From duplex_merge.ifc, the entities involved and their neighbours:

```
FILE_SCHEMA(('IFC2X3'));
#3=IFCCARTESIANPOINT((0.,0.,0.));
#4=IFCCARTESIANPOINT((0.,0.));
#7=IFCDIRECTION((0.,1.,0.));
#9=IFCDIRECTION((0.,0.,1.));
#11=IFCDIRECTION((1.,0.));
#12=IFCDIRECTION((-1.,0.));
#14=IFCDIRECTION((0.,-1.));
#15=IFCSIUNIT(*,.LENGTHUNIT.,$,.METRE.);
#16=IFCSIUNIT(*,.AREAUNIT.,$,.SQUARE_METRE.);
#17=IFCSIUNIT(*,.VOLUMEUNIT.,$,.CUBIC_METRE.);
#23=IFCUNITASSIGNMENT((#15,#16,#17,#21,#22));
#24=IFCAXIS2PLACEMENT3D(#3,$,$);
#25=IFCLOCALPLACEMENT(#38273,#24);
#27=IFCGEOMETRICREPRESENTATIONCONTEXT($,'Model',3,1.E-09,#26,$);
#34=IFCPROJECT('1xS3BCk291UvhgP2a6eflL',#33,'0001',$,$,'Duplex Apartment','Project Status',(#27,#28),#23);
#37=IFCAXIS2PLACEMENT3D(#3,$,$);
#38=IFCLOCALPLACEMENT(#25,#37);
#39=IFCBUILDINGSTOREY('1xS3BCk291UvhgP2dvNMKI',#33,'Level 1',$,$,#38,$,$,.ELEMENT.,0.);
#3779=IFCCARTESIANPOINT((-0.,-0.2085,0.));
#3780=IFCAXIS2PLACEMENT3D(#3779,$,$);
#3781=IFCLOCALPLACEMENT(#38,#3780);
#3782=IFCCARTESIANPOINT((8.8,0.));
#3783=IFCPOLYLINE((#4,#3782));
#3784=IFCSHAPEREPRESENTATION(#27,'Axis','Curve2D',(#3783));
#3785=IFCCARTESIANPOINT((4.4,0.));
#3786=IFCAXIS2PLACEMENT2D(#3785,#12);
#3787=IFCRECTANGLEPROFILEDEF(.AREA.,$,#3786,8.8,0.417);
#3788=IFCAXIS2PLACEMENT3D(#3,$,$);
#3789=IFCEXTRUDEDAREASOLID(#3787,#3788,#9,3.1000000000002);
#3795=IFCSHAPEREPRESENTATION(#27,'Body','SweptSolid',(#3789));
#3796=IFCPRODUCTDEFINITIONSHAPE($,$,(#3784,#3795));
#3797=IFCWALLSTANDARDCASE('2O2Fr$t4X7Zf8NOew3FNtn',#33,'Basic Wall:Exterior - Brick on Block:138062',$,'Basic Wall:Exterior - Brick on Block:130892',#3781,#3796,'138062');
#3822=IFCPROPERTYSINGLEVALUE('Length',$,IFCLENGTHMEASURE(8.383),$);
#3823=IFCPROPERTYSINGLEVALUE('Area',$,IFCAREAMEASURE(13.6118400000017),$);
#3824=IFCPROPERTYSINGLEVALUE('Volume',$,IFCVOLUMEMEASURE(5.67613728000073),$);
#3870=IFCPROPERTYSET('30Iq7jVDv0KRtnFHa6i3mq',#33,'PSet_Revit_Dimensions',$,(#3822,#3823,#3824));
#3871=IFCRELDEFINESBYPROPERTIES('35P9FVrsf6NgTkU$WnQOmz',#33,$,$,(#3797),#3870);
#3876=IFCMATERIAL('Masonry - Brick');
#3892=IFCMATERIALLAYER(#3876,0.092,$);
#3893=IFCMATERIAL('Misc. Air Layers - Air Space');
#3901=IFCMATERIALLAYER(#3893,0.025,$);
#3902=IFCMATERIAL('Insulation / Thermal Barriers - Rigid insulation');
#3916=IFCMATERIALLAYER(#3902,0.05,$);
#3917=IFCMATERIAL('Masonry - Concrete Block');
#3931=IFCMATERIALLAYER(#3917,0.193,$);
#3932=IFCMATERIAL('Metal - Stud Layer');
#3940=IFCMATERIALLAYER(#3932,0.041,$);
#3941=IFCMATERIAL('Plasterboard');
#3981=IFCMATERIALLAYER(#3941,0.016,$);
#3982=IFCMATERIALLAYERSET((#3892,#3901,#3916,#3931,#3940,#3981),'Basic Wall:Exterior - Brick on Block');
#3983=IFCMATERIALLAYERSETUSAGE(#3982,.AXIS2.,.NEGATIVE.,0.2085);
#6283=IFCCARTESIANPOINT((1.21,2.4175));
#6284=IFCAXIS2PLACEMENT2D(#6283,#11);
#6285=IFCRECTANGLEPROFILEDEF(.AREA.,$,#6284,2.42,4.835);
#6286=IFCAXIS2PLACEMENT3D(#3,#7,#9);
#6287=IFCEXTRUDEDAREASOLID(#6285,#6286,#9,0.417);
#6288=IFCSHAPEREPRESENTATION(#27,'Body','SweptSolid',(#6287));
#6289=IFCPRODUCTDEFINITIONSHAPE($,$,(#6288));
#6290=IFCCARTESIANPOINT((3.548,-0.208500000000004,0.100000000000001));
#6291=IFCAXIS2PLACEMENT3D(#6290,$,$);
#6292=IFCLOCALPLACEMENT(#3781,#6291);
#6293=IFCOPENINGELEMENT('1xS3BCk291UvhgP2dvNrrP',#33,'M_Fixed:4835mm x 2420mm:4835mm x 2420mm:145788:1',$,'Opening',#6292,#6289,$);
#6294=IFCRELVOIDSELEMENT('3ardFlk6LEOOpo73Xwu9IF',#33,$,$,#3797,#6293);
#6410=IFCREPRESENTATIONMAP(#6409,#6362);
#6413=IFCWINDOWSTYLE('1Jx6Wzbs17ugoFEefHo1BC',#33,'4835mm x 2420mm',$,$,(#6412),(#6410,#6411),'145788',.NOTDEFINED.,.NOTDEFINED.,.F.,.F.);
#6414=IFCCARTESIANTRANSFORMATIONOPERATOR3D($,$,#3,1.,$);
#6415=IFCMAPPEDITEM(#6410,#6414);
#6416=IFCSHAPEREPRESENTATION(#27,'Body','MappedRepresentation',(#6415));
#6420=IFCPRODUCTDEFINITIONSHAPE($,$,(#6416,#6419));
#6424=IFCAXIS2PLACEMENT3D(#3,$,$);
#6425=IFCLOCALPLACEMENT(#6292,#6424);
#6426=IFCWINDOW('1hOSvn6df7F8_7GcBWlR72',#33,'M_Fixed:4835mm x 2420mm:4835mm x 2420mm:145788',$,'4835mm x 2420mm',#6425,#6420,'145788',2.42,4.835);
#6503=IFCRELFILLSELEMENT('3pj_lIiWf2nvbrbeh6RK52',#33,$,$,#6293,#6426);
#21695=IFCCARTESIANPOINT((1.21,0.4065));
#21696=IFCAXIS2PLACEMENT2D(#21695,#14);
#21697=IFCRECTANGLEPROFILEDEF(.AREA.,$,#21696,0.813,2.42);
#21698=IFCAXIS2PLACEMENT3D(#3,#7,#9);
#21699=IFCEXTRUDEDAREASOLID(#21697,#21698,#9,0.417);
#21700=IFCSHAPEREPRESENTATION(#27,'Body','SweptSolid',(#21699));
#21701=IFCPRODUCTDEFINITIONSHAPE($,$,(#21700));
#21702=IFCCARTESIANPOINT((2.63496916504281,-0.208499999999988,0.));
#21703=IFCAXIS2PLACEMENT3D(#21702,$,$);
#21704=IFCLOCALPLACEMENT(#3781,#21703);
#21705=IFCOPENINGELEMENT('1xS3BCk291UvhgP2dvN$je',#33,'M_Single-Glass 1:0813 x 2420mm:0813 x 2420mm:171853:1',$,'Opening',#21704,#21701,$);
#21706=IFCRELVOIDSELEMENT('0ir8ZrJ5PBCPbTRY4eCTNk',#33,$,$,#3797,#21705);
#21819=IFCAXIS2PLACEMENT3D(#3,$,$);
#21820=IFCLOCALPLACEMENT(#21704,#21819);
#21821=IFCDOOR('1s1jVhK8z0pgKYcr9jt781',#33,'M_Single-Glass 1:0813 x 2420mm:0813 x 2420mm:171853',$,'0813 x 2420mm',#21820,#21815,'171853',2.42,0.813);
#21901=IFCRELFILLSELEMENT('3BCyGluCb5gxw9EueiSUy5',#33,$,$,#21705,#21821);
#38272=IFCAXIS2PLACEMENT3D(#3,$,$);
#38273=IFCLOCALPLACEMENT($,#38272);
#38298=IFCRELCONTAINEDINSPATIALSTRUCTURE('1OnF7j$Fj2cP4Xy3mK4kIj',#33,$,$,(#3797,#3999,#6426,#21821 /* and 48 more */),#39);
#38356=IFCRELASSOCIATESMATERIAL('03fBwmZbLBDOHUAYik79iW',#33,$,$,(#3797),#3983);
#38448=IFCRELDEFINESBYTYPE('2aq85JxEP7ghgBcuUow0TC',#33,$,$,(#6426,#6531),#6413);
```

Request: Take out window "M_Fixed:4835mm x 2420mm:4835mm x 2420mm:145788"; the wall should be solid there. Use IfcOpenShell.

```python
import ifcopenshell
import ifcopenshell.api.feature
import ifcopenshell.api.pset
import ifcopenshell.api.root
import ifcopenshell.geom
import ifcopenshell.util.element
import ifcopenshell.util.shape
import ifcopenshell.util.unit

model = ifcopenshell.open("duplex_merge.ifc")
area_scale = ifcopenshell.util.unit.calculate_unit_scale(model, "AREAUNIT")
volume_scale = ifcopenshell.util.unit.calculate_unit_scale(model, "VOLUMEUNIT")
settings = ifcopenshell.geom.settings()


def volume(element):
    """Net volume in cubic metres, openings subtracted."""
    shape = ifcopenshell.geom.create_shape(settings, element)
    return ifcopenshell.util.shape.get_volume(shape.geometry)


window = model.by_guid("1hOSvn6df7F8_7GcBWlR72")
opening = window.FillsVoids[0].RelatingOpeningElement
wall = opening.VoidsElements[0].RelatingBuildingElement
before = volume(wall)

ifcopenshell.api.root.remove_product(model, product=window)
ifcopenshell.api.feature.remove_feature(model, feature=opening)

after = volume(wall)
thickness = 0.417  # wall thickness in metres

# Update the wall's stored quantities.
pset = model.by_id(ifcopenshell.util.element.get_pset(wall, "PSet_Revit_Dimensions", should_inherit=False)["id"])
ifcopenshell.api.pset.edit_pset(model, pset=pset, properties={
    "Area": model.create_entity("IfcAreaMeasure", after / thickness / area_scale),
    "Volume": model.create_entity("IfcVolumeMeasure", after / volume_scale),
})

print(f"wall volume {before:.3f} -> {after:.3f} m3")

model.write("duplex_merge-out.ifc")
```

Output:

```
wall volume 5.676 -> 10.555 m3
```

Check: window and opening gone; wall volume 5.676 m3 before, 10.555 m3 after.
